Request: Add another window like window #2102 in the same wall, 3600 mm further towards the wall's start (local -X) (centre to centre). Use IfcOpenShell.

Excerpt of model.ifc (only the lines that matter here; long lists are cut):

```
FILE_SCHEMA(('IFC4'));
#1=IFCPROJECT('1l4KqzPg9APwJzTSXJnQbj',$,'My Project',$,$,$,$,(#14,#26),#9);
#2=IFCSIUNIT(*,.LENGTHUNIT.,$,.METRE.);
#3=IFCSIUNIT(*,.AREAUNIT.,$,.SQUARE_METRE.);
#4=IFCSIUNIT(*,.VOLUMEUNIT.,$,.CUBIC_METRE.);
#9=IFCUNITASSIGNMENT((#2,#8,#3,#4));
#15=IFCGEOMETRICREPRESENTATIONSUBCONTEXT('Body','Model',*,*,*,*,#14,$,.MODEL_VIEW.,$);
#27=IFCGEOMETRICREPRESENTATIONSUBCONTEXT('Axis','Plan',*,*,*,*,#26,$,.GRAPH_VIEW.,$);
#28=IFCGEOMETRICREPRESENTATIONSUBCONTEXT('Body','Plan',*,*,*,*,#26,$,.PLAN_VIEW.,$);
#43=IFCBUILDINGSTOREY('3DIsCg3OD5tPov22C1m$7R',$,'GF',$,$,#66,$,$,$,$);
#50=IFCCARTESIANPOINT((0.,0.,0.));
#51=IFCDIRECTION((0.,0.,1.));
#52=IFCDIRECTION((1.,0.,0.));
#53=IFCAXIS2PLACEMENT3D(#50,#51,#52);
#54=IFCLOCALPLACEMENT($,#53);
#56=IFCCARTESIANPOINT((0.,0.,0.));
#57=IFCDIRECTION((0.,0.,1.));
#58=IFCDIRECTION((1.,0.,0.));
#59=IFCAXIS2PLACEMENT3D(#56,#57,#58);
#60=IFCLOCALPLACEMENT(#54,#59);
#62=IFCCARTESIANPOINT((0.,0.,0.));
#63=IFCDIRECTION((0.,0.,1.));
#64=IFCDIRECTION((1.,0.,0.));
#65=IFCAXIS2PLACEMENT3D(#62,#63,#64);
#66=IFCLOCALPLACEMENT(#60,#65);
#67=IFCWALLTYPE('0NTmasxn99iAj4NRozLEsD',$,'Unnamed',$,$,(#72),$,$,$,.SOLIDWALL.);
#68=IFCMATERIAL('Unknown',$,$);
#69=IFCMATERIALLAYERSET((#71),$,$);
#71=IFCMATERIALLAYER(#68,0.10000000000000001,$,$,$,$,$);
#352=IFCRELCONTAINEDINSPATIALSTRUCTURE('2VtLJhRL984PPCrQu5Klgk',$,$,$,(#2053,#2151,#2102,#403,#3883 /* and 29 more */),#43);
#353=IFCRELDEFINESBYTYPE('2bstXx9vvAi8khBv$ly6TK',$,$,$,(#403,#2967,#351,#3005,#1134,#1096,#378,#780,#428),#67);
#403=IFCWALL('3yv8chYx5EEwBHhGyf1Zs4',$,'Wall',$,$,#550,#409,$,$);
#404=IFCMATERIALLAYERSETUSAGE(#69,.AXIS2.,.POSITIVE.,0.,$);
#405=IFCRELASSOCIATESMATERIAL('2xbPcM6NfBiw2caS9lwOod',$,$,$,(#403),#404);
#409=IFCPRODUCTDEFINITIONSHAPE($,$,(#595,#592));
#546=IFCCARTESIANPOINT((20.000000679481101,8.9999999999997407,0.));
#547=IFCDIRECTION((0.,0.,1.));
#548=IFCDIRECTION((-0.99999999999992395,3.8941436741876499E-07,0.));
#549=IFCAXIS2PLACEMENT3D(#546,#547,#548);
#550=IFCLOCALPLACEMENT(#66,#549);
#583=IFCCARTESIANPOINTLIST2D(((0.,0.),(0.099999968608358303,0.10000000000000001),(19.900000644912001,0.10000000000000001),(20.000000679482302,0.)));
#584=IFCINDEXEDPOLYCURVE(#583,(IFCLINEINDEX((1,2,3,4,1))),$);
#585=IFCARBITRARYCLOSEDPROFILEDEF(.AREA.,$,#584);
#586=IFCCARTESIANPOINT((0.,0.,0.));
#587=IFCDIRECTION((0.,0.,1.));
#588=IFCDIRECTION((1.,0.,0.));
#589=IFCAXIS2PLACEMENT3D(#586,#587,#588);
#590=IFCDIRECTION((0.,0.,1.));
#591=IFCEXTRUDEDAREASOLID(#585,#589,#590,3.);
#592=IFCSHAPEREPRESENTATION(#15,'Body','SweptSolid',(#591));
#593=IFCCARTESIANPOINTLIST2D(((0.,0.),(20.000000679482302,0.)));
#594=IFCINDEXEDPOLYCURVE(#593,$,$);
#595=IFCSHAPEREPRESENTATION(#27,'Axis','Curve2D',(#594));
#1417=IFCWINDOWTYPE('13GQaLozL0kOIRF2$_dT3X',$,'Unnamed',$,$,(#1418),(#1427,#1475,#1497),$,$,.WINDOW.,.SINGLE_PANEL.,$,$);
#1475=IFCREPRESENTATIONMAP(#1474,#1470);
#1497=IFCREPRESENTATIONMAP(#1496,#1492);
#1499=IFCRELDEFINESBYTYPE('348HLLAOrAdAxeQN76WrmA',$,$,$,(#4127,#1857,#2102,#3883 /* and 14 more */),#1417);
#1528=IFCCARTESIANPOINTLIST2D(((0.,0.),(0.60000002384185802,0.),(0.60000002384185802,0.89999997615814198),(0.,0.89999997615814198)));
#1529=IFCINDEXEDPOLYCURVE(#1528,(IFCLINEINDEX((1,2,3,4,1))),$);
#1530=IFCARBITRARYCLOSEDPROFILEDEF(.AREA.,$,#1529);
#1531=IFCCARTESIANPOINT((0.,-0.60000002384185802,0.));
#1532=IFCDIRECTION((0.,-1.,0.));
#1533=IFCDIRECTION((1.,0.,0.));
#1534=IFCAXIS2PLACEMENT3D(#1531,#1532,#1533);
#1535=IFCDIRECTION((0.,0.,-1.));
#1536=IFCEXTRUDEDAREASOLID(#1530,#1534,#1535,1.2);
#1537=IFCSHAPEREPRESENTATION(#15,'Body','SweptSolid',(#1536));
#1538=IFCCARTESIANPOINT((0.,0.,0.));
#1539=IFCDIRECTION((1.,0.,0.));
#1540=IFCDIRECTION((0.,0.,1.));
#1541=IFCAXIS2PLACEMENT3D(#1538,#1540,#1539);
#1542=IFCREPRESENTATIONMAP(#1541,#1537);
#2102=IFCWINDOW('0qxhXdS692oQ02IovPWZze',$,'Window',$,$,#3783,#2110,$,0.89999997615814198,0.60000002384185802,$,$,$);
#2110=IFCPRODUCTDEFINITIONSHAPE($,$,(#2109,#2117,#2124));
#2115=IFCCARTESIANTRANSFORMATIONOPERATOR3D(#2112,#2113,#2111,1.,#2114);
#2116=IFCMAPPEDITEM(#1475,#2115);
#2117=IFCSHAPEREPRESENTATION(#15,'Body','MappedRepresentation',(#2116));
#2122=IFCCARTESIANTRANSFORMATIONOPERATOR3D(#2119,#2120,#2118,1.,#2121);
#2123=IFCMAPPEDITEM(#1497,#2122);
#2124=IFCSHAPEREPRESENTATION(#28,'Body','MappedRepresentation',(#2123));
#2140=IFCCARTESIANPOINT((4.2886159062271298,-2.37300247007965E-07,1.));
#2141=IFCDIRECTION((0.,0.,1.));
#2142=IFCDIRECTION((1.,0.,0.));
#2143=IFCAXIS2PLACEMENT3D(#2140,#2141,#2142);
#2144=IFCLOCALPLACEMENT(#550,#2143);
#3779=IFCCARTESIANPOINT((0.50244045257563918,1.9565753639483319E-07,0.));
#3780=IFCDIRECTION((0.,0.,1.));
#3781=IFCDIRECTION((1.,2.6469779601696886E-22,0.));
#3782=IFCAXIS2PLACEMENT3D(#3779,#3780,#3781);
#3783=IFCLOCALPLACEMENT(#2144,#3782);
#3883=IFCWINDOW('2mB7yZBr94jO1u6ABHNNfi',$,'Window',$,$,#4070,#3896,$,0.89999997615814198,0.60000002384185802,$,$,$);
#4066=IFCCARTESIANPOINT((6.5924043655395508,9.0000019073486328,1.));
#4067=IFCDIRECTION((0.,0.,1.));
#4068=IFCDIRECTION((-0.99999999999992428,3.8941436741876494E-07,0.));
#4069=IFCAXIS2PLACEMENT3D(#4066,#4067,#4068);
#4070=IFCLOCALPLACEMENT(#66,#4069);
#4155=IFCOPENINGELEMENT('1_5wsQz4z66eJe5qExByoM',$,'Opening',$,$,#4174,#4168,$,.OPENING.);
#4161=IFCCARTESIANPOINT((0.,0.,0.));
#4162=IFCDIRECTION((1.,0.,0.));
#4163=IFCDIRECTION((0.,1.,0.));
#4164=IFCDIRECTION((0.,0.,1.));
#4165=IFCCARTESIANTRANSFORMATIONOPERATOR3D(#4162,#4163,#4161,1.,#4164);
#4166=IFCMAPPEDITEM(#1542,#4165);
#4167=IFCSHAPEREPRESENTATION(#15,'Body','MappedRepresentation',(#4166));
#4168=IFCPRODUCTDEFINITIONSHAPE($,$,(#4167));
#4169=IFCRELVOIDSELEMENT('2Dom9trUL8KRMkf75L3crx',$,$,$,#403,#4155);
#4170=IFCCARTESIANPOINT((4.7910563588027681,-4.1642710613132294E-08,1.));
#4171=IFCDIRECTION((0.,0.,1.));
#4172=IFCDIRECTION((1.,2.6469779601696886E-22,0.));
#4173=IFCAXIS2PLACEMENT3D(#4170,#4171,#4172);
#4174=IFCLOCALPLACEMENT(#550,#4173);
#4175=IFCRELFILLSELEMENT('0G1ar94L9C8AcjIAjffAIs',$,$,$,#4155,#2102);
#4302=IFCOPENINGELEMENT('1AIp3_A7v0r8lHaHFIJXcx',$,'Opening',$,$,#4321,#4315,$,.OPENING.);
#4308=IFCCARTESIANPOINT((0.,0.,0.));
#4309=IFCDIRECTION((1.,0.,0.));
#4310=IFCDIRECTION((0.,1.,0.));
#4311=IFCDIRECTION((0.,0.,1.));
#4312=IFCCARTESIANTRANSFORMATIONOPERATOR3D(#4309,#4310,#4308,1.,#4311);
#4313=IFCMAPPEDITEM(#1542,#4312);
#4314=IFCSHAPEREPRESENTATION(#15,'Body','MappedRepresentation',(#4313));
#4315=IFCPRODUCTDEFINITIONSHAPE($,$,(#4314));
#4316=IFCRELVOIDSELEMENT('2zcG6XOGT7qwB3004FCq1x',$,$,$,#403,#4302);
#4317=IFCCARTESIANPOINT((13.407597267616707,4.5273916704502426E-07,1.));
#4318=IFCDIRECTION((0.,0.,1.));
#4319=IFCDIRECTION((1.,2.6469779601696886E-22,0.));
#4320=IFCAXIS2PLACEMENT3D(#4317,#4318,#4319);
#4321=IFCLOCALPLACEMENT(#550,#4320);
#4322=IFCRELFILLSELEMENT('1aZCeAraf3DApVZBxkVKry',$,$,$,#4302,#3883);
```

```python
import ifcopenshell
import ifcopenshell.api.feature
import ifcopenshell.api.geometry
import ifcopenshell.api.root
import ifcopenshell.geom
import ifcopenshell.util.element
import ifcopenshell.util.placement
import ifcopenshell.util.shape
import ifcopenshell.util.unit

model = ifcopenshell.open("model.ifc")
unit_scale = ifcopenshell.util.unit.calculate_unit_scale(model)
settings = ifcopenshell.geom.settings()


def volume(element):
    """Net volume in cubic metres, openings subtracted."""
    shape = ifcopenshell.geom.create_shape(settings, element)
    return ifcopenshell.util.shape.get_volume(shape.geometry)


window = model.by_guid("0qxhXdS692oQ02IovPWZze")
opening = window.FillsVoids[0].RelatingOpeningElement
wall = opening.VoidsElements[0].RelatingBuildingElement
before = volume(wall)
shift = ifcopenshell.util.placement.get_local_placement(wall.ObjectPlacement)[:3, 0] * -3.6 / unit_scale

# copy_class copies the void relationship, type, container and properties, but no geometry.
new_opening = ifcopenshell.api.root.copy_class(model, product=opening)
new_opening.Representation = ifcopenshell.util.element.copy_deep(
    model, opening.Representation, exclude=["IfcGeometricRepresentationContext", "IfcRepresentationMap"]
)
new_window = ifcopenshell.api.root.copy_class(model, product=window)
new_window.Representation = ifcopenshell.util.element.copy_deep(
    model, window.Representation, exclude=["IfcGeometricRepresentationContext", "IfcRepresentationMap"]
)
ifcopenshell.api.feature.add_filling(model, opening=new_opening, element=new_window)

for old, new in ((opening, new_opening), (window, new_window)):
    matrix = ifcopenshell.util.placement.get_local_placement(old.ObjectPlacement)
    matrix[:3, 3] += shift
    ifcopenshell.api.geometry.edit_object_placement(model, product=new, matrix=matrix, is_si=False)

after = volume(wall)

print(f"wall volume {before:.3f} -> {after:.3f} m3")

model.write("model_v2.ifc")
```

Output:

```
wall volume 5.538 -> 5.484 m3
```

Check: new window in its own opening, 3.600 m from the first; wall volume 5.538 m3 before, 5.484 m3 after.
